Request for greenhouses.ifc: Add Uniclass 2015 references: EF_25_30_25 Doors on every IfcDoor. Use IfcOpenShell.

First a look at what the model holds.

```python
import ifcopenshell

model = ifcopenshell.open("greenhouses.ifc")
print(model.schema)
print("classifications:", [c.Name for c in model.by_type("IfcClassification")])
for ifc_class in ("IfcDoor", "IfcRoof", "IfcStair", "IfcWall", "IfcWindow"):
    print(ifc_class, len(model.by_type(ifc_class)))
```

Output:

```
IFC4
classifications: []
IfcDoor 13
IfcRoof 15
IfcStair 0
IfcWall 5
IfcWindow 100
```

```python
import ifcopenshell
import ifcopenshell.api.classification

model = ifcopenshell.open("greenhouses.ifc")

system = ifcopenshell.api.classification.add_classification(model, classification="Uniclass 2015")

codes = {
    "IfcDoor": ("EF_25_30_25", "Doors"),
}
for ifc_class, (code, name) in codes.items():
    products = model.by_type(ifc_class)
    ifcopenshell.api.classification.add_reference(
        model, products=products, classification=system, identification=code, name=name
    )
    print(code, len(products))

model.write("greenhouses_rev.ifc")
```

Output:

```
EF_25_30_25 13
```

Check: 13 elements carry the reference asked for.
